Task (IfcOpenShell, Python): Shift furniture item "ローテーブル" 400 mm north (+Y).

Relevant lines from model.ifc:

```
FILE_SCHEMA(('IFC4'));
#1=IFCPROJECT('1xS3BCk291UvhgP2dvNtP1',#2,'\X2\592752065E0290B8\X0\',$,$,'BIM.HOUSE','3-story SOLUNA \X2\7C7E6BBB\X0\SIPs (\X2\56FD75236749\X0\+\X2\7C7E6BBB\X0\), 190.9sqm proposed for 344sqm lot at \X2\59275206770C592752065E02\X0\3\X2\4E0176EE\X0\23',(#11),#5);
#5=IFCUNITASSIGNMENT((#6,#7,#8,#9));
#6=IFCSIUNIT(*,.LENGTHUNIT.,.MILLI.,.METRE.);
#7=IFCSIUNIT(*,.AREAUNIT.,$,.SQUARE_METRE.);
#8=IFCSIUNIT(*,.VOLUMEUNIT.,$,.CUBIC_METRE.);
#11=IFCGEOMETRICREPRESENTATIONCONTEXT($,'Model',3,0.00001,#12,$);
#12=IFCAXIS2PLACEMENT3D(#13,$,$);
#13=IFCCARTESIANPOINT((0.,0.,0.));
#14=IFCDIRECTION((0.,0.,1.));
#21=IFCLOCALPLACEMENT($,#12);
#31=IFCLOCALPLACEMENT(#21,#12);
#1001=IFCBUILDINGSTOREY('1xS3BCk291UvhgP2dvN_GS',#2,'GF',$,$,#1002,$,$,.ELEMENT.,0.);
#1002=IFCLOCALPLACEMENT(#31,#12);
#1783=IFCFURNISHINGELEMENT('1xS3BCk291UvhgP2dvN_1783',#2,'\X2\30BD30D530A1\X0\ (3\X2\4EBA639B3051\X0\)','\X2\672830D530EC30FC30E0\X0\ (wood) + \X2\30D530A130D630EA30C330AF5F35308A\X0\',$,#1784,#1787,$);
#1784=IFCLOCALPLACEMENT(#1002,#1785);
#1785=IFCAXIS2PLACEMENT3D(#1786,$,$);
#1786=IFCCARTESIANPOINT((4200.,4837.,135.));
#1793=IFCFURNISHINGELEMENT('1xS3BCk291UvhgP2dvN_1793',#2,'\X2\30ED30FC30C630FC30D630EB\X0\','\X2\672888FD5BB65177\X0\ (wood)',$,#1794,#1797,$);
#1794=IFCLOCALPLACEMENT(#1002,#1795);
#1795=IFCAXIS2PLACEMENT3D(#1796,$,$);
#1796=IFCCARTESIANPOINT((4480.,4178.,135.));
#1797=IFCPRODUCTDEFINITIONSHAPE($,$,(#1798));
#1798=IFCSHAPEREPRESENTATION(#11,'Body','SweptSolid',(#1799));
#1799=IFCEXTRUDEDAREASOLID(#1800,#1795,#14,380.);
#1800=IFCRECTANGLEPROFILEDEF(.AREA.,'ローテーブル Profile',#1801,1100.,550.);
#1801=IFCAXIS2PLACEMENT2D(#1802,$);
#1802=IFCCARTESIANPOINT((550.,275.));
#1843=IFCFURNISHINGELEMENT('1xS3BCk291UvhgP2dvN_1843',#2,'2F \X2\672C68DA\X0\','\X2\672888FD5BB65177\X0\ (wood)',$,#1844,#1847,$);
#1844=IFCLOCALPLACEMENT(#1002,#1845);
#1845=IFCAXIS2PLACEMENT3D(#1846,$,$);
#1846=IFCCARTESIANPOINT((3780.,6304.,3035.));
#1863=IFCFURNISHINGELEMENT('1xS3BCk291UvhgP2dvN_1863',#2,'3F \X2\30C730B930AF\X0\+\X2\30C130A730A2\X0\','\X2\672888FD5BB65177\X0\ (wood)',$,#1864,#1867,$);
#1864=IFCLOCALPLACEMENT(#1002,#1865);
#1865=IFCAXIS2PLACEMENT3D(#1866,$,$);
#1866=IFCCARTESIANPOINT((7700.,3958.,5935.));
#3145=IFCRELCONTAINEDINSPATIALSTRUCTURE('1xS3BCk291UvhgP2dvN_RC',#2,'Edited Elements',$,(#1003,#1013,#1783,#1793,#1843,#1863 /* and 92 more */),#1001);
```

```python
import ifcopenshell
import ifcopenshell.api.geometry
import ifcopenshell.util.placement

model = ifcopenshell.open("model.ifc")

item = model.by_guid("1xS3BCk291UvhgP2dvN_1793")
matrix = ifcopenshell.util.placement.get_local_placement(item.ObjectPlacement)
matrix[1, 3] += 400.0
ifcopenshell.api.geometry.edit_object_placement(model, product=item, matrix=matrix, is_si=False)

print(ifcopenshell.util.placement.get_local_placement(item.ObjectPlacement).round(3) + 0.0)

model.write("model_updated.ifc")
```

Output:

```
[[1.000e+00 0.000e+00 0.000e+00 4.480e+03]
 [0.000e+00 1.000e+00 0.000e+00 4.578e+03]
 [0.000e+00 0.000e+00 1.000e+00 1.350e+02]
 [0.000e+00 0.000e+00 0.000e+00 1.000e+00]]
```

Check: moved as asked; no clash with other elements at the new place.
